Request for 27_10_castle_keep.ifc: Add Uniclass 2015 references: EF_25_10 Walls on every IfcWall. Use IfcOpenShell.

First a look at what the model holds.

```python
import ifcopenshell

model = ifcopenshell.open("27_10_castle_keep.ifc")
print(model.schema)
print("classifications:", [c.Name for c in model.by_type("IfcClassification")])
for ifc_class in ("IfcDoor", "IfcRoof", "IfcStair", "IfcWall", "IfcWindow"):
    print(ifc_class, len(model.by_type(ifc_class)))
```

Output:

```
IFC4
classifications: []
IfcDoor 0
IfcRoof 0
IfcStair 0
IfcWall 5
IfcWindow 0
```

```python
import ifcopenshell
import ifcopenshell.api.classification

model = ifcopenshell.open("27_10_castle_keep.ifc")

system = ifcopenshell.api.classification.add_classification(model, classification="Uniclass 2015")

codes = {
    "IfcWall": ("EF_25_10", "Walls"),
}
for ifc_class, (code, name) in codes.items():
    products = model.by_type(ifc_class)
    ifcopenshell.api.classification.add_reference(
        model, products=products, classification=system, identification=code, name=name
    )
    print(code, len(products))

model.write("27_10_castle_keep_rev.ifc")
```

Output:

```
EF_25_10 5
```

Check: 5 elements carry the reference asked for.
